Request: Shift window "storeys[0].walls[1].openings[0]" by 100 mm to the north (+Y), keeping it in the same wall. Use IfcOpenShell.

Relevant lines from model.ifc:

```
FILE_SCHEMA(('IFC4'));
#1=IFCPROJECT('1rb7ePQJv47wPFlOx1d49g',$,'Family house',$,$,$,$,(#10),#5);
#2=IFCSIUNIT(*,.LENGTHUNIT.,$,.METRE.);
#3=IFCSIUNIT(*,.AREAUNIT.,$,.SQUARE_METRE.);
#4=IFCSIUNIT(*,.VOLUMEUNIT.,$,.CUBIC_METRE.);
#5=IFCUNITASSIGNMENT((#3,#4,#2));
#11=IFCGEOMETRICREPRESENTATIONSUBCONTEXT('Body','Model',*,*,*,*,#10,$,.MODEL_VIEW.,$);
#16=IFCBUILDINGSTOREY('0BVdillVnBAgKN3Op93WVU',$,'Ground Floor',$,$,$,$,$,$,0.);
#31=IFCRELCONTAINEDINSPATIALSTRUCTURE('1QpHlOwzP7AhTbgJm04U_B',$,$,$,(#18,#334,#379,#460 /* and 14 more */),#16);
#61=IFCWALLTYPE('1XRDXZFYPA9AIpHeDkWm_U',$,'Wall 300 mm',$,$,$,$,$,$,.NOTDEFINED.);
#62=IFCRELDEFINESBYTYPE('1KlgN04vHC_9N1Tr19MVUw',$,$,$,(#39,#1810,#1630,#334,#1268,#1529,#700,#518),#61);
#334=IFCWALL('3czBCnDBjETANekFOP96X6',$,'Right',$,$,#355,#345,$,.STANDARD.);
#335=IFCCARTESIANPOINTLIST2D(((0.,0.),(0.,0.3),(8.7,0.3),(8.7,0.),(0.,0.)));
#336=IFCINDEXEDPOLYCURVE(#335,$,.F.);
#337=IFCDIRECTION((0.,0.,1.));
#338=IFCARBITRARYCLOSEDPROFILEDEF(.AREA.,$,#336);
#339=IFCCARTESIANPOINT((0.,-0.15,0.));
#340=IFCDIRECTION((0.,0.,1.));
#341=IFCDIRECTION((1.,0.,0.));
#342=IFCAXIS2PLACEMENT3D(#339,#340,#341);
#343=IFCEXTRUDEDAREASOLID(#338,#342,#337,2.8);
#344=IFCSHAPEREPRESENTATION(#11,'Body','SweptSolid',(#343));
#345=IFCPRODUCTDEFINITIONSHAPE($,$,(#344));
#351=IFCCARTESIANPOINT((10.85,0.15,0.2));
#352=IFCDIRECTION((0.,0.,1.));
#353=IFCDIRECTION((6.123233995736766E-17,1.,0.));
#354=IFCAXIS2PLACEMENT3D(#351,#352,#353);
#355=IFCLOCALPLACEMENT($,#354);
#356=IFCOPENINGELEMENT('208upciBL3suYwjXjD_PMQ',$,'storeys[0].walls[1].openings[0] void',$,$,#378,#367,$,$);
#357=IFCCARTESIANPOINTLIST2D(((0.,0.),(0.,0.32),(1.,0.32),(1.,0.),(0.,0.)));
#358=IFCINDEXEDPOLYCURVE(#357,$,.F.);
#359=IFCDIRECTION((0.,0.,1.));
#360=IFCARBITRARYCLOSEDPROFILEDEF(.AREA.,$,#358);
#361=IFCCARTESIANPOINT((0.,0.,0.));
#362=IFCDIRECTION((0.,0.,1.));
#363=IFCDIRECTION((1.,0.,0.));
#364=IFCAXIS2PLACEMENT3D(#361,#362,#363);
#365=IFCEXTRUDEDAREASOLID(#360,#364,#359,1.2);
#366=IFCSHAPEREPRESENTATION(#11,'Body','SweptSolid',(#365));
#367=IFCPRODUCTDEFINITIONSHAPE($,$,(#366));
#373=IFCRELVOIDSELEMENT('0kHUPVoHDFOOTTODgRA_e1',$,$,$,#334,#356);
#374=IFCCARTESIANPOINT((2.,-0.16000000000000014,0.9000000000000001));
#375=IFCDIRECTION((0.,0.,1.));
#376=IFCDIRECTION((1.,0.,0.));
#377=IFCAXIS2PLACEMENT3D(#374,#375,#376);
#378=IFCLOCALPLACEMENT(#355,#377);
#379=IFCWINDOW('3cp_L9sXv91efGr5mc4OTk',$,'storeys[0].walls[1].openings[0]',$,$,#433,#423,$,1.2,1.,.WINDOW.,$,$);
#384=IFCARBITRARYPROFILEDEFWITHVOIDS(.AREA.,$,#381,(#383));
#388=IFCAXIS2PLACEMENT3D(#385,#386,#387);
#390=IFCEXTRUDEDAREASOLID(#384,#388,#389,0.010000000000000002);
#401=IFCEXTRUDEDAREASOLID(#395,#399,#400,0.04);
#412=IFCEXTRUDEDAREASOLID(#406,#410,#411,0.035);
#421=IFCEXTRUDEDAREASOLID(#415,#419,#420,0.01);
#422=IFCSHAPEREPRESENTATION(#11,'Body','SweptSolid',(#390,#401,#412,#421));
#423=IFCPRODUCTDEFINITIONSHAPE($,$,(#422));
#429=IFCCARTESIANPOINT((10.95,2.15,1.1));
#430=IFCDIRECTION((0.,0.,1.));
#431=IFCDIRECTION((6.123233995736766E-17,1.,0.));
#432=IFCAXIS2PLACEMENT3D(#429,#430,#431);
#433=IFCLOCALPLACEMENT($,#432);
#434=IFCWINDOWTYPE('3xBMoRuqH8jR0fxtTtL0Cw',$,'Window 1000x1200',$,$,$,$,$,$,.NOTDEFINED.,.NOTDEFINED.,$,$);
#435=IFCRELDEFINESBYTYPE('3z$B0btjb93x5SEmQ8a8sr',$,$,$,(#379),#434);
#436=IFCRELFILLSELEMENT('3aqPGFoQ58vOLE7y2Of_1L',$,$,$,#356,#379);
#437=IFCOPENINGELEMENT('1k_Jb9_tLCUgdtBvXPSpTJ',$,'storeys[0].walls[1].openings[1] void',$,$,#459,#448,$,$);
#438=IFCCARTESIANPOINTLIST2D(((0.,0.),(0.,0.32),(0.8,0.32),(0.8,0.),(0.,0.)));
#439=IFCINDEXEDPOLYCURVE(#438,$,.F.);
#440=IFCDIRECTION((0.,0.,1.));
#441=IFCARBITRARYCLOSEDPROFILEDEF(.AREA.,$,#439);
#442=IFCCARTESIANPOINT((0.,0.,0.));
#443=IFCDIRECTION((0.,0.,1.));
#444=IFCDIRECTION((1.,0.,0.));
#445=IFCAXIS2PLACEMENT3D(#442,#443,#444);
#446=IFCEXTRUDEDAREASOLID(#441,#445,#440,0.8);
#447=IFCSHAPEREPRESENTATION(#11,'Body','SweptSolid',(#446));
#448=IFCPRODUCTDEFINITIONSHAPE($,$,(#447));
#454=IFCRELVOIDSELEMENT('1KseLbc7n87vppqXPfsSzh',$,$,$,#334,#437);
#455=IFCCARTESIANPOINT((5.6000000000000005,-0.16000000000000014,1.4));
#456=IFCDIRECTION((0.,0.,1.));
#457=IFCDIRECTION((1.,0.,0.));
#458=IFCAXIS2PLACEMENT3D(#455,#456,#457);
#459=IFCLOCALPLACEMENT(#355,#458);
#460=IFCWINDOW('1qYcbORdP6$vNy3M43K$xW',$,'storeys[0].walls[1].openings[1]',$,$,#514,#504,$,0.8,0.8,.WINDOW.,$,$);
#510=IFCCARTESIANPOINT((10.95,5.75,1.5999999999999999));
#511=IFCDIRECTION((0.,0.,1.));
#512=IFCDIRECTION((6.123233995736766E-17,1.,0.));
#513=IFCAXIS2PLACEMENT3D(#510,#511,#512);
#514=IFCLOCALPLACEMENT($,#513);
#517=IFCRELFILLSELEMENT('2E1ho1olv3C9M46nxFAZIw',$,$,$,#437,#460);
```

```python
import ifcopenshell
import ifcopenshell.api.geometry
import ifcopenshell.util.placement
import ifcopenshell.util.unit

model = ifcopenshell.open("model.ifc")
unit_scale = ifcopenshell.util.unit.calculate_unit_scale(model)

window = model.by_guid("3cp_L9sXv91efGr5mc4OTk")
opening = window.FillsVoids[0].RelatingOpeningElement
wall = opening.VoidsElements[0].RelatingBuildingElement

wall_matrix = ifcopenshell.util.placement.get_local_placement(wall.ObjectPlacement)
shift = wall_matrix[:3, 0] * 0.1 / unit_scale
before = ifcopenshell.util.placement.get_local_placement(window.ObjectPlacement)[:3, 3].copy()

# The window is not placed relative to its opening, so move both.
for product in (opening, window):
    matrix = ifcopenshell.util.placement.get_local_placement(product.ObjectPlacement)
    matrix[:3, 3] += shift
    ifcopenshell.api.geometry.edit_object_placement(model, product=product, matrix=matrix, is_si=False)

after = ifcopenshell.util.placement.get_local_placement(window.ObjectPlacement)[:3, 3]
print("window moved by", (after - before).round(3) + 0.0)

model.write("model-out.ifc")
```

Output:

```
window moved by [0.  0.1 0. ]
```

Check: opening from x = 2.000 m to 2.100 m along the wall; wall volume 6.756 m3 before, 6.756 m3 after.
